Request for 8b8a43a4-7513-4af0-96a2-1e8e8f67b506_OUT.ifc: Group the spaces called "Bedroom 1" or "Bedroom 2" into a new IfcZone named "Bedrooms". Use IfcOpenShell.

First a look at what the model holds.

```python
import ifcopenshell

model = ifcopenshell.open("8b8a43a4-7513-4af0-96a2-1e8e8f67b506_OUT.ifc")
print(model.schema)
seen = {}
for space in model.by_type("IfcSpace"):
    seen[space.LongName] = seen.get(space.LongName, 0) + 1
for name, count in sorted(seen.items(), key=str):
    print(count, "x", name)
print("zones:", [z.Name for z in model.by_type("IfcZone")][:20])
```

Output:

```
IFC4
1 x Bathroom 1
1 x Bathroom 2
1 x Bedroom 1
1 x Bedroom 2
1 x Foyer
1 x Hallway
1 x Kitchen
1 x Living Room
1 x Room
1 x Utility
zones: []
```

```python
import ifcopenshell
import ifcopenshell.api.group
import ifcopenshell.api.root

model = ifcopenshell.open("8b8a43a4-7513-4af0-96a2-1e8e8f67b506_OUT.ifc")

names = {"Bedroom 1", "Bedroom 2"}
spaces = [s for s in model.by_type("IfcSpace") if s.LongName in names]

zone = ifcopenshell.api.root.create_entity(model, ifc_class="IfcZone", name="Bedrooms")
ifcopenshell.api.group.assign_group(model, products=spaces, group=zone)
print(len(spaces), "spaces in", zone.Name)

model.write("8b8a43a4-7513-4af0-96a2-1e8e8f67b506_OUT_rev.ifc")
```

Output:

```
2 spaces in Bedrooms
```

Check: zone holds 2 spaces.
